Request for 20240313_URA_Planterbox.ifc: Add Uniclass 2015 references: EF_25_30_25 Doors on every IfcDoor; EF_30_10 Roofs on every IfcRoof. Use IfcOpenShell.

First a look at what the model holds.

```python
import ifcopenshell

model = ifcopenshell.open("20240313_URA_Planterbox.ifc")
print(model.schema)
print("classifications:", [c.Name for c in model.by_type("IfcClassification")])
for ifc_class in ("IfcDoor", "IfcRoof", "IfcStair", "IfcWall", "IfcWindow"):
    print(ifc_class, len(model.by_type(ifc_class)))
```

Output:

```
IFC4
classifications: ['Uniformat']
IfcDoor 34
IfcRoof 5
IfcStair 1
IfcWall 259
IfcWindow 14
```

```python
import ifcopenshell
import ifcopenshell.api.classification

model = ifcopenshell.open("20240313_URA_Planterbox.ifc")

system = ifcopenshell.api.classification.add_classification(model, classification="Uniclass 2015")

codes = {
    "IfcDoor": ("EF_25_30_25", "Doors"),
    "IfcRoof": ("EF_30_10", "Roofs"),
}
for ifc_class, (code, name) in codes.items():
    products = model.by_type(ifc_class)
    ifcopenshell.api.classification.add_reference(
        model, products=products, classification=system, identification=code, name=name
    )
    print(code, len(products))

model.write("20240313_URA_Planterbox_updated.ifc")
```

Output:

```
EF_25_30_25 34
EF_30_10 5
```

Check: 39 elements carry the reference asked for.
